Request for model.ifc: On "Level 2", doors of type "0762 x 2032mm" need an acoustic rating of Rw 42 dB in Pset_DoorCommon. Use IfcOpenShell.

First a look at what the model holds.

```python
import ifcopenshell
import ifcopenshell.util.element

model = ifcopenshell.open("model.ifc")
print(model.schema)
storey = next(s for s in model.by_type("IfcBuildingStorey") if s.Name == "Level 2")
doors = [e for e in ifcopenshell.util.element.get_decomposition(storey) if e.is_a("IfcDoor")]
seen = {}
for e in doors:
    element_type = ifcopenshell.util.element.get_type(e)
    key = (element_type.Name if element_type != e and element_type else None, ifcopenshell.util.element.get_pset(e, "Pset_DoorCommon", "AcousticRating"))
    seen[key] = seen.get(key, 0) + 1
for (name, value), count in sorted(seen.items(), key=str):
    print(count, "x", name, "|", value)
```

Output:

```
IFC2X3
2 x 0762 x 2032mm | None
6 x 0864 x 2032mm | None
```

```python
import ifcopenshell
import ifcopenshell.api.pset
import ifcopenshell.util.element

model = ifcopenshell.open("model.ifc")

storey = next(s for s in model.by_type("IfcBuildingStorey") if s.Name == "Level 2")
doors = [e for e in ifcopenshell.util.element.get_decomposition(storey) if e.is_a("IfcDoor")]

count = 0
for e in doors:
    element_type = ifcopenshell.util.element.get_type(e)
    if element_type in (None, e) or element_type.Name != "0762 x 2032mm":
        continue
    # add_pset returns the element's existing set when there is one.
    pset = ifcopenshell.api.pset.add_pset(model, product=e, name="Pset_DoorCommon")
    ifcopenshell.api.pset.edit_pset(model, pset=pset, properties={"AcousticRating": "Rw 42 dB"})
    count += 1

print(count, "doors updated")

model.write("model-out.ifc")
```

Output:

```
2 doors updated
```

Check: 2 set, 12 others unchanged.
